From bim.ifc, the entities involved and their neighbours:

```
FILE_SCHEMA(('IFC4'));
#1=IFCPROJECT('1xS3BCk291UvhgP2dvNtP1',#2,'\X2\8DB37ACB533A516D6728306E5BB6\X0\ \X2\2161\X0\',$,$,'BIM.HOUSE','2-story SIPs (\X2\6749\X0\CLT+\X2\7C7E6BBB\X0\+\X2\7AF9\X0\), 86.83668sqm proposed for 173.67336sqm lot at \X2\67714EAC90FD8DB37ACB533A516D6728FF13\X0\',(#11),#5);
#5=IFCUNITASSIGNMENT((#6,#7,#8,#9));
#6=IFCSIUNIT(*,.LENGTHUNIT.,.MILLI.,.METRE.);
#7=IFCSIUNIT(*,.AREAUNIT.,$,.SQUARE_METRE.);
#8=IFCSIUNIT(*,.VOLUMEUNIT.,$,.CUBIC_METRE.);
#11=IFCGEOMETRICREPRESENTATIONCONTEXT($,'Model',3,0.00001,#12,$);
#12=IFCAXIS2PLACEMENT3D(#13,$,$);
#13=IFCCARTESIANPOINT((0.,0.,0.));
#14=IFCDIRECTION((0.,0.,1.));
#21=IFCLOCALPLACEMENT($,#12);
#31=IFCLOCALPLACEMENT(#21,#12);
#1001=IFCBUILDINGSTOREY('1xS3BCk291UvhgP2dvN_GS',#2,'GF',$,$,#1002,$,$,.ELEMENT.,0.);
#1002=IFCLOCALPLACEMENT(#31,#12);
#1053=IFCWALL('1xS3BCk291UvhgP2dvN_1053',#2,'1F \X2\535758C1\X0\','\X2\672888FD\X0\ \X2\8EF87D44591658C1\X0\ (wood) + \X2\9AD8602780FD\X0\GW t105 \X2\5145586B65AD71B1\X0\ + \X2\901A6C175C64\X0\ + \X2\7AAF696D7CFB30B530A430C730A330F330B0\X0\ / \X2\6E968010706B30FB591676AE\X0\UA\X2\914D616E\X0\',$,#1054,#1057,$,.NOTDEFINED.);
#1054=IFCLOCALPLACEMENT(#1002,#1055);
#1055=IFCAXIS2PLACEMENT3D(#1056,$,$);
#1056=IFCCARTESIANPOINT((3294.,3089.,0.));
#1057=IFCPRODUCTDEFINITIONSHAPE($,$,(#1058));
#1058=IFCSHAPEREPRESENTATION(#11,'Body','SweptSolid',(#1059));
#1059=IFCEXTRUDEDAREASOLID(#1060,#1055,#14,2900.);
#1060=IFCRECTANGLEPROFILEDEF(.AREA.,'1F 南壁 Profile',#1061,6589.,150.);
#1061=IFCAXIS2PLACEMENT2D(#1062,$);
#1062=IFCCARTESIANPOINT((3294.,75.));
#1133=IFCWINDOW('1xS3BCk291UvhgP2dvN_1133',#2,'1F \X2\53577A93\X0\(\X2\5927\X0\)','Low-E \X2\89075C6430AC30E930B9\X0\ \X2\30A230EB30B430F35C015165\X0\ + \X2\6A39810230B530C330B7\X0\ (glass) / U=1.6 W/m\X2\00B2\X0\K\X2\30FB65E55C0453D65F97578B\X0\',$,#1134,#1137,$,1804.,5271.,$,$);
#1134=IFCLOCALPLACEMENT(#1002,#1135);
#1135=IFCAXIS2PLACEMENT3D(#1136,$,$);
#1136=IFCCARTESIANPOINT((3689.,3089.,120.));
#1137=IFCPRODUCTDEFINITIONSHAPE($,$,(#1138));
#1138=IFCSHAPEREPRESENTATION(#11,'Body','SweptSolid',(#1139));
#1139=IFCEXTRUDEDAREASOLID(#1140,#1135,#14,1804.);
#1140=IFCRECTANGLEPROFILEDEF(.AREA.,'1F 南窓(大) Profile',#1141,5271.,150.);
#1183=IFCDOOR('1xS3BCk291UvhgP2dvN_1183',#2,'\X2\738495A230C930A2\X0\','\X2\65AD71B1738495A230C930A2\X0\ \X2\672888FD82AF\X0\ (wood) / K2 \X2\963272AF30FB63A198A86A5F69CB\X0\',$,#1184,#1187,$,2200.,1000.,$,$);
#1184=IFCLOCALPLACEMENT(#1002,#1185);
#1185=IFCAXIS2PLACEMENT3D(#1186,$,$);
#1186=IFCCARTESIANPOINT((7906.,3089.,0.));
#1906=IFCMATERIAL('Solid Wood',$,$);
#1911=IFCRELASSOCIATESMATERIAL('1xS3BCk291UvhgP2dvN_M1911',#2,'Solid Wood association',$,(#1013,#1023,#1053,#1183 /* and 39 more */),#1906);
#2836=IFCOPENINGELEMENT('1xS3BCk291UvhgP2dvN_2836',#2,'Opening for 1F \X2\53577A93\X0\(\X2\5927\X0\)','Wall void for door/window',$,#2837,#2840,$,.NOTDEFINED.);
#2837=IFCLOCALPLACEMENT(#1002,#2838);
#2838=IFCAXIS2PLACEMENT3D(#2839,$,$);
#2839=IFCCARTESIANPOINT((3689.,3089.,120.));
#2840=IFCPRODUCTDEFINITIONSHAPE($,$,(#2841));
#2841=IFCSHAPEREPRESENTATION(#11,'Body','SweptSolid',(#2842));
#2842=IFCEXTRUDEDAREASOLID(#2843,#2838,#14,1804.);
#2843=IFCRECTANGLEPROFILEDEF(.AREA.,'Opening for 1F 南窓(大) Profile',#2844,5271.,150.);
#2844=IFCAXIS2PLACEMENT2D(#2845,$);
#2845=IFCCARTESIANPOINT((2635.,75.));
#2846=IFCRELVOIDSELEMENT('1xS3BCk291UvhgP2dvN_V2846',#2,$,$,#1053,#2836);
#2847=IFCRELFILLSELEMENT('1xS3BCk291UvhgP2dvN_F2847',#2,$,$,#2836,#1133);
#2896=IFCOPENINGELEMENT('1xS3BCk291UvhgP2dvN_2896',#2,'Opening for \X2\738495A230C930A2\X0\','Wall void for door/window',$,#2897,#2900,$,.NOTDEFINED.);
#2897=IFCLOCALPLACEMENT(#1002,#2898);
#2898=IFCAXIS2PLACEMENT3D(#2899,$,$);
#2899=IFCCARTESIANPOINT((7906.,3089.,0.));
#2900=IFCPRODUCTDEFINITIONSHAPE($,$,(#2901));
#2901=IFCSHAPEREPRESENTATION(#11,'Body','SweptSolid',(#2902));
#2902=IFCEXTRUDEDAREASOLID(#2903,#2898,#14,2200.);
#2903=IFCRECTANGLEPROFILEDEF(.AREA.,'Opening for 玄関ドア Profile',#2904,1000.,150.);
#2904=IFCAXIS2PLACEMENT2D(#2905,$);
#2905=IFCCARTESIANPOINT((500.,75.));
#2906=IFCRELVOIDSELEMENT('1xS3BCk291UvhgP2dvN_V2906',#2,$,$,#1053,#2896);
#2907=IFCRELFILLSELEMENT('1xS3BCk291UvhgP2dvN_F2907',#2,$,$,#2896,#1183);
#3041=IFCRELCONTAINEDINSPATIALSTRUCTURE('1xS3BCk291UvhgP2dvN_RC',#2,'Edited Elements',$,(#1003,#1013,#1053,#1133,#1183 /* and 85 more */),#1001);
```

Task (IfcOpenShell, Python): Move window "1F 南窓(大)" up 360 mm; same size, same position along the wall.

```python
import numpy as np
import ifcopenshell
import ifcopenshell.api.geometry
import ifcopenshell.util.placement
import ifcopenshell.util.unit

model = ifcopenshell.open("bim.ifc")
unit_scale = ifcopenshell.util.unit.calculate_unit_scale(model)

window = model.by_guid("1xS3BCk291UvhgP2dvN_1133")
opening = window.FillsVoids[0].RelatingOpeningElement
dz = 0.36 / unit_scale

shift = np.array([0.0, 0.0, dz])
# The window is not placed relative to its opening, so move both.
for product in (opening, window):
    matrix = ifcopenshell.util.placement.get_local_placement(product.ObjectPlacement)
    matrix[:3, 3] += shift
    ifcopenshell.api.geometry.edit_object_placement(model, product=product, matrix=matrix, is_si=False)

print(f"moved by {dz * unit_scale:+.3f} m")

model.write("bim_rev.ifc")
```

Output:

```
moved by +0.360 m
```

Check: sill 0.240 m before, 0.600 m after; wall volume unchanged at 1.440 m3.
